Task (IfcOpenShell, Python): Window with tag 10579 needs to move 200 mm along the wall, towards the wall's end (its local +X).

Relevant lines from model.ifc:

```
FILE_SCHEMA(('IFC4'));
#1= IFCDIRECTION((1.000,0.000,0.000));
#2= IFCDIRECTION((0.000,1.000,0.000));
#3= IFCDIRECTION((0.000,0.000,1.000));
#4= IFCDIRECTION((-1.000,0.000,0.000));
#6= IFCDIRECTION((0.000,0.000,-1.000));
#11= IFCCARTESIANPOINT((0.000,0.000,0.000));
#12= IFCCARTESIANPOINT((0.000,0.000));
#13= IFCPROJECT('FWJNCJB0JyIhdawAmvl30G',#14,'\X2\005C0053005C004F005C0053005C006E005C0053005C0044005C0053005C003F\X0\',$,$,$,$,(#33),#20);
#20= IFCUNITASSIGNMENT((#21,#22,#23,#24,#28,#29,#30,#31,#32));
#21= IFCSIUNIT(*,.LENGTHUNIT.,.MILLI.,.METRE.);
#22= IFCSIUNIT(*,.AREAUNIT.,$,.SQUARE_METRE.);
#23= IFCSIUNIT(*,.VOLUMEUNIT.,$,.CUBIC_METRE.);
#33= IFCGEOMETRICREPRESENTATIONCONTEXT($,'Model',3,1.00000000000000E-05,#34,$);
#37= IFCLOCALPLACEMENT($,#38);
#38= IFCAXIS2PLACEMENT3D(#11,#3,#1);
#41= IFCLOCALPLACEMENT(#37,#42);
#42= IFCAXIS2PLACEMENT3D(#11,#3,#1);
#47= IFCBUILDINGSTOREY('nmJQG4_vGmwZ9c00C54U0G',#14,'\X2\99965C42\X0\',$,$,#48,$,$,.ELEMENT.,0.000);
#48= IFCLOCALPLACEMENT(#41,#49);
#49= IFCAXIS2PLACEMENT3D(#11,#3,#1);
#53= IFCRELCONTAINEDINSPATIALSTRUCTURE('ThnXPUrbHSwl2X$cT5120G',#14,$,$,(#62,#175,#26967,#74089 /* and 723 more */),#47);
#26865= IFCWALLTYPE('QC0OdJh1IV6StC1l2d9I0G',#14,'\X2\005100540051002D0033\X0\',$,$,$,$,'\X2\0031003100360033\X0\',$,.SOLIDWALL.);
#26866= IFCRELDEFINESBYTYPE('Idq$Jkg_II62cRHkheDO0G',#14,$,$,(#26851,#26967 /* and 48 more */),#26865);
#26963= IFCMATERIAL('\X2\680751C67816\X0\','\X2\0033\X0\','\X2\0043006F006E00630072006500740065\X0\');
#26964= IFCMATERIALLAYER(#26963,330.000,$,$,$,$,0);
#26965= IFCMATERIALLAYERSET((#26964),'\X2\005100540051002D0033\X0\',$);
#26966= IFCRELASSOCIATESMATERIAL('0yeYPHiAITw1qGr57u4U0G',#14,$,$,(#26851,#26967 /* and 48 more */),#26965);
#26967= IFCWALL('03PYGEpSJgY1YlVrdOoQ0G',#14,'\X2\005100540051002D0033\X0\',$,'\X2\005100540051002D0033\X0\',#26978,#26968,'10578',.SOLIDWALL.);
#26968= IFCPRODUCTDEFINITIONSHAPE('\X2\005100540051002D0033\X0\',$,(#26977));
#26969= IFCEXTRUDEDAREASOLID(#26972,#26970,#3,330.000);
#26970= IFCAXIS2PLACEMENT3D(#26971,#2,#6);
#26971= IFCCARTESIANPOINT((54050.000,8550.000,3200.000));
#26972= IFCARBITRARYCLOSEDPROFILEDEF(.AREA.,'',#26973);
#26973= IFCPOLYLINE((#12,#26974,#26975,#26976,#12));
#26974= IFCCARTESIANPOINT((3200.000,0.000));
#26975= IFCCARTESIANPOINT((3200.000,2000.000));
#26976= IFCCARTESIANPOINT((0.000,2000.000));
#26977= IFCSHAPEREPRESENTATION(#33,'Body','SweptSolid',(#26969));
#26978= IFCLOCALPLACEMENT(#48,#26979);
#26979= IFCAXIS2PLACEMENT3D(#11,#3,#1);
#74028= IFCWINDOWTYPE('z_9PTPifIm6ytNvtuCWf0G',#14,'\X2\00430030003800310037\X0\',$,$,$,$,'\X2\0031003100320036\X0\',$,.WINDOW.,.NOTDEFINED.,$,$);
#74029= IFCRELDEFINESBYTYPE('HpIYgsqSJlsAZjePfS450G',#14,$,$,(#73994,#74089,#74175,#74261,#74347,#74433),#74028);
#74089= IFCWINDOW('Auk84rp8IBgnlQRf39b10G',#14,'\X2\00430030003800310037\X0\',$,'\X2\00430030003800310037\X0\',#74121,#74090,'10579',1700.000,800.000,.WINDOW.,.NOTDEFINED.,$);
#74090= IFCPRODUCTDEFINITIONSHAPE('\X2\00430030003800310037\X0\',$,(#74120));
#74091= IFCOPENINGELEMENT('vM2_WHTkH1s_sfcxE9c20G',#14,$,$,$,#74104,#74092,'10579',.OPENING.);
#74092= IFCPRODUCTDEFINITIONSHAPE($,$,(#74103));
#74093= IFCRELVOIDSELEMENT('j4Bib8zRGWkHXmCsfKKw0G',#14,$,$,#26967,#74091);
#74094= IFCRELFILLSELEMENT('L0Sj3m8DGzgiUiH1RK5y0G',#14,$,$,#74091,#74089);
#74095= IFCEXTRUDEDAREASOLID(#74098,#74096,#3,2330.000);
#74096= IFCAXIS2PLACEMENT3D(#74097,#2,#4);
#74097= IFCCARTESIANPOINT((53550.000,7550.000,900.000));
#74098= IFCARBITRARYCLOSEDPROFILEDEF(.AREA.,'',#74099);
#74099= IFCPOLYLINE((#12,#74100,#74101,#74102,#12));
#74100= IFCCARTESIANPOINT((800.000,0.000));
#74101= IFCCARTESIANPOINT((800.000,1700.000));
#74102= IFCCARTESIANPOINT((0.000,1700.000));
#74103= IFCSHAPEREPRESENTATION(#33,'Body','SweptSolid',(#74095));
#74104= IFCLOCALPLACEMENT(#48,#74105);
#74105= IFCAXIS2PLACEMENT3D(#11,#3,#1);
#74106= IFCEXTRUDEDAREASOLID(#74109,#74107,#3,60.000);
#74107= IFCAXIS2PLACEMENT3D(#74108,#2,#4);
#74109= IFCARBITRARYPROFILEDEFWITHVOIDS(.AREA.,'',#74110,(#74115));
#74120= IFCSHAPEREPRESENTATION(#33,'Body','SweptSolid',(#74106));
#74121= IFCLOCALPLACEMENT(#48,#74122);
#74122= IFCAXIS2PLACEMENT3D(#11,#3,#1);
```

```python
import ifcopenshell
import ifcopenshell.api.geometry
import ifcopenshell.util.placement
import ifcopenshell.util.unit

model = ifcopenshell.open("model.ifc")
unit_scale = ifcopenshell.util.unit.calculate_unit_scale(model)

window = model.by_id(74089)
opening = window.FillsVoids[0].RelatingOpeningElement
wall = opening.VoidsElements[0].RelatingBuildingElement

wall_matrix = ifcopenshell.util.placement.get_local_placement(wall.ObjectPlacement)
shift = wall_matrix[:3, 0] * 0.2 / unit_scale
before = ifcopenshell.util.placement.get_local_placement(window.ObjectPlacement)[:3, 3].copy()

# The window is not placed relative to its opening, so move both.
for product in (opening, window):
    matrix = ifcopenshell.util.placement.get_local_placement(product.ObjectPlacement)
    matrix[:3, 3] += shift
    ifcopenshell.api.geometry.edit_object_placement(model, product=product, matrix=matrix, is_si=False)

after = ifcopenshell.util.placement.get_local_placement(window.ObjectPlacement)[:3, 3]
print("window moved by", (after - before).round(3) + 0.0)

model.write("model_edited.ifc")
```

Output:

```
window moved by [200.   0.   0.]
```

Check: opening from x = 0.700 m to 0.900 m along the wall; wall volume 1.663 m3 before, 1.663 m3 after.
